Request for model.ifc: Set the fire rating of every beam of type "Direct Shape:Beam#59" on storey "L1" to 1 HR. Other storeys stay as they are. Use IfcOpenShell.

First a look at what the model holds.

```python
import ifcopenshell
import ifcopenshell.util.element

model = ifcopenshell.open("model.ifc")
print(model.schema)
storey = next(s for s in model.by_type("IfcBuildingStorey") if s.Name == "L1")
beams = [e for e in ifcopenshell.util.element.get_decomposition(storey) if e.is_a("IfcBeam")]
seen = {}
for e in beams:
    element_type = ifcopenshell.util.element.get_type(e)
    key = (element_type.Name if element_type != e and element_type else None, ifcopenshell.util.element.get_pset(e, "Pset_BeamCommon", "FireRating"))
    seen[key] = seen.get(key, 0) + 1
for (name, value), count in sorted(seen.items(), key=str):
    print(count, "x", name, "|", value)
```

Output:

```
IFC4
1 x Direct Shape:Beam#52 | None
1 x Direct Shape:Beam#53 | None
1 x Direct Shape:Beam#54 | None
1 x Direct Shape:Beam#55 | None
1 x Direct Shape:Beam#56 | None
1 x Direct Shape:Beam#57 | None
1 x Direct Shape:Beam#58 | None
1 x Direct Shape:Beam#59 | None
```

```python
import ifcopenshell
import ifcopenshell.api.pset
import ifcopenshell.util.element

model = ifcopenshell.open("model.ifc")

storey = next(s for s in model.by_type("IfcBuildingStorey") if s.Name == "L1")
beams = [e for e in ifcopenshell.util.element.get_decomposition(storey) if e.is_a("IfcBeam")]

count = 0
for e in beams:
    element_type = ifcopenshell.util.element.get_type(e)
    if element_type in (None, e) or element_type.Name != "Direct Shape:Beam#59":
        continue
    # add_pset returns the element's existing set when there is one.
    pset = ifcopenshell.api.pset.add_pset(model, product=e, name="Pset_BeamCommon")
    ifcopenshell.api.pset.edit_pset(model, pset=pset, properties={"FireRating": "1 HR"})
    count += 1

print(count, "beams updated")

model.write("model_updated.ifc")
```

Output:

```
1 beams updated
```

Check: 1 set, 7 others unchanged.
